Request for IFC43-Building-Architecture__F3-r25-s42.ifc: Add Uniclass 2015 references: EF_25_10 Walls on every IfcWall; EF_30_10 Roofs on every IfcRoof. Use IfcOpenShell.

First a look at what the model holds.

```python
import ifcopenshell

model = ifcopenshell.open("IFC43-Building-Architecture__F3-r25-s42.ifc")
print(model.schema)
print("classifications:", [c.Name for c in model.by_type("IfcClassification")])
for ifc_class in ("IfcDoor", "IfcRoof", "IfcStair", "IfcWall", "IfcWindow"):
    print(ifc_class, len(model.by_type(ifc_class)))
```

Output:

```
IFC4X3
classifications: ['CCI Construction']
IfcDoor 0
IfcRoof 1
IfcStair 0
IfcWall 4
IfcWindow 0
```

```python
import ifcopenshell
import ifcopenshell.api.classification

model = ifcopenshell.open("IFC43-Building-Architecture__F3-r25-s42.ifc")

system = ifcopenshell.api.classification.add_classification(model, classification="Uniclass 2015")

codes = {
    "IfcWall": ("EF_25_10", "Walls"),
    "IfcRoof": ("EF_30_10", "Roofs"),
}
for ifc_class, (code, name) in codes.items():
    products = model.by_type(ifc_class)
    ifcopenshell.api.classification.add_reference(
        model, products=products, classification=system, identification=code, name=name
    )
    print(code, len(products))

model.write("IFC43-Building-Architecture__F3-r25-s42_updated.ifc")
```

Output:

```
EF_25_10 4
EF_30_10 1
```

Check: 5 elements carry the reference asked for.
